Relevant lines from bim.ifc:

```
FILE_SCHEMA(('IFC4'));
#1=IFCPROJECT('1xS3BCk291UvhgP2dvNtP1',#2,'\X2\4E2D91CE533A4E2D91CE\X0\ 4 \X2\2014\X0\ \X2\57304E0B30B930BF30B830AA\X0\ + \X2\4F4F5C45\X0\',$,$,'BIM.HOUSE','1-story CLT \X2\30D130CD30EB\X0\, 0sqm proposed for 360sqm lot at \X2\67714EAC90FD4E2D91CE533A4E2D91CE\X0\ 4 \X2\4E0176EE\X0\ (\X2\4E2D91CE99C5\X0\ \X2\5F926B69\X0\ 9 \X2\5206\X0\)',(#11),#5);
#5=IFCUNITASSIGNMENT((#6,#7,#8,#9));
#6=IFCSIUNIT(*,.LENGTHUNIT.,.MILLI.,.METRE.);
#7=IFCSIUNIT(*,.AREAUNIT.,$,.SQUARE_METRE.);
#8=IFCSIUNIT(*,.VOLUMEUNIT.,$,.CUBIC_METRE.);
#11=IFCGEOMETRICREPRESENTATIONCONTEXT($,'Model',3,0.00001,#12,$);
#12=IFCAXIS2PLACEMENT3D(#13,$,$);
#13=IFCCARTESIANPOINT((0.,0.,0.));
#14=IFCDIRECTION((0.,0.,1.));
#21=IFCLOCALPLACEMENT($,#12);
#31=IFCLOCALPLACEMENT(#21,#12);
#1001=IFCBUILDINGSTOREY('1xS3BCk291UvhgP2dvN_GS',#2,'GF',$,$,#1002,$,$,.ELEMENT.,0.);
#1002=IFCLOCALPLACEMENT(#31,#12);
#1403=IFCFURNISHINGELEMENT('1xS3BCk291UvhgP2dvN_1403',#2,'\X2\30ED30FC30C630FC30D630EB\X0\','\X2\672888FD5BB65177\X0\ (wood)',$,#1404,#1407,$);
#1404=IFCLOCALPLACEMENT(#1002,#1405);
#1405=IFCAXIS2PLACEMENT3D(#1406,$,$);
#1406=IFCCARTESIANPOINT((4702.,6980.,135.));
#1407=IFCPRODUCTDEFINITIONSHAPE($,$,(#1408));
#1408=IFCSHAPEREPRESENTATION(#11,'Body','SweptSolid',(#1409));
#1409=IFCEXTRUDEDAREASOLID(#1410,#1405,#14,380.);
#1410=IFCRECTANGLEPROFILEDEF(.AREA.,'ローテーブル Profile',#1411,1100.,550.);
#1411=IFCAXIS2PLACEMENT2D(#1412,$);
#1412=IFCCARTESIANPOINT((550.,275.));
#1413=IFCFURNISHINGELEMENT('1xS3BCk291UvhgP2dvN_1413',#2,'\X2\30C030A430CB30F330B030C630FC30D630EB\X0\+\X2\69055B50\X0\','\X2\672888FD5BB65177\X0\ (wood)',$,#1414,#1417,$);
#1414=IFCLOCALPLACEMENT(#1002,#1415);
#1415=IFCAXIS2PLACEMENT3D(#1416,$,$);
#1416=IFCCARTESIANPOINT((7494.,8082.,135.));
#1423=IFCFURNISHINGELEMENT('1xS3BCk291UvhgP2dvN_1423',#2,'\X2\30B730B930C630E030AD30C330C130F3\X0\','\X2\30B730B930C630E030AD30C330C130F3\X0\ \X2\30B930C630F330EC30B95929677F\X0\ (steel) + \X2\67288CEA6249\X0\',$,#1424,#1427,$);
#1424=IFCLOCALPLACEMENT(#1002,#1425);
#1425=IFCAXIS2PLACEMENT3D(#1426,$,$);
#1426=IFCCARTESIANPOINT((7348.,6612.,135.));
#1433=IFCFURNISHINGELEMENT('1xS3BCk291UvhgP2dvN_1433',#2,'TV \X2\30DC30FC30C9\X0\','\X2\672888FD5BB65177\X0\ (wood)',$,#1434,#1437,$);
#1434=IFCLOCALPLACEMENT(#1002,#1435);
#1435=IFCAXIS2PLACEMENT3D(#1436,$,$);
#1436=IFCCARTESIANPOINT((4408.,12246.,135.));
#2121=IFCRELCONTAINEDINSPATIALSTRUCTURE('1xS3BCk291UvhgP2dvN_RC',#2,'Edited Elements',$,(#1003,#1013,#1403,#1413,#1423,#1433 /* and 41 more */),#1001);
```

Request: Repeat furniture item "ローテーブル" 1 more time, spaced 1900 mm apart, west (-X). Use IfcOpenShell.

```python
import numpy as np
import ifcopenshell
import ifcopenshell.api.geometry
import ifcopenshell.api.root
import ifcopenshell.util.element
import ifcopenshell.util.placement

model = ifcopenshell.open("bim.ifc")


def reuse_history(source, copy):
    """copy_class also copies each property set's owner history, people and application; keep the originals."""
    for rel in copy.IsDefinedBy:
        if rel.is_a("IfcRelDefinesByProperties") and (history := rel.RelatingPropertyDefinition.OwnerHistory):
            rel.RelatingPropertyDefinition.OwnerHistory = source.OwnerHistory
            ifcopenshell.util.element.remove_deep2(model, history)


source = model.by_guid("1xS3BCk291UvhgP2dvN_1403")
base = ifcopenshell.util.placement.get_local_placement(source.ObjectPlacement)
step = np.array([-1.0, 0.0, 0.0]) * 1900.0

for i in range(1, 2):
    copy = ifcopenshell.api.root.copy_class(model, product=source)
    copy.Representation = ifcopenshell.util.element.copy_deep(
        model, source.Representation, exclude=["IfcGeometricRepresentationContext", "IfcRepresentationMap"]
    )
    reuse_history(source, copy)
    matrix = base.copy()
    matrix[:3, 3] += i * step
    print("added at", matrix[:3, 3].round(3) + 0.0)
    ifcopenshell.api.geometry.edit_object_placement(model, product=copy, matrix=matrix, is_si=False)

model.write("bim_rev.ifc")
```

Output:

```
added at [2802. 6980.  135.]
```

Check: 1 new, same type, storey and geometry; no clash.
